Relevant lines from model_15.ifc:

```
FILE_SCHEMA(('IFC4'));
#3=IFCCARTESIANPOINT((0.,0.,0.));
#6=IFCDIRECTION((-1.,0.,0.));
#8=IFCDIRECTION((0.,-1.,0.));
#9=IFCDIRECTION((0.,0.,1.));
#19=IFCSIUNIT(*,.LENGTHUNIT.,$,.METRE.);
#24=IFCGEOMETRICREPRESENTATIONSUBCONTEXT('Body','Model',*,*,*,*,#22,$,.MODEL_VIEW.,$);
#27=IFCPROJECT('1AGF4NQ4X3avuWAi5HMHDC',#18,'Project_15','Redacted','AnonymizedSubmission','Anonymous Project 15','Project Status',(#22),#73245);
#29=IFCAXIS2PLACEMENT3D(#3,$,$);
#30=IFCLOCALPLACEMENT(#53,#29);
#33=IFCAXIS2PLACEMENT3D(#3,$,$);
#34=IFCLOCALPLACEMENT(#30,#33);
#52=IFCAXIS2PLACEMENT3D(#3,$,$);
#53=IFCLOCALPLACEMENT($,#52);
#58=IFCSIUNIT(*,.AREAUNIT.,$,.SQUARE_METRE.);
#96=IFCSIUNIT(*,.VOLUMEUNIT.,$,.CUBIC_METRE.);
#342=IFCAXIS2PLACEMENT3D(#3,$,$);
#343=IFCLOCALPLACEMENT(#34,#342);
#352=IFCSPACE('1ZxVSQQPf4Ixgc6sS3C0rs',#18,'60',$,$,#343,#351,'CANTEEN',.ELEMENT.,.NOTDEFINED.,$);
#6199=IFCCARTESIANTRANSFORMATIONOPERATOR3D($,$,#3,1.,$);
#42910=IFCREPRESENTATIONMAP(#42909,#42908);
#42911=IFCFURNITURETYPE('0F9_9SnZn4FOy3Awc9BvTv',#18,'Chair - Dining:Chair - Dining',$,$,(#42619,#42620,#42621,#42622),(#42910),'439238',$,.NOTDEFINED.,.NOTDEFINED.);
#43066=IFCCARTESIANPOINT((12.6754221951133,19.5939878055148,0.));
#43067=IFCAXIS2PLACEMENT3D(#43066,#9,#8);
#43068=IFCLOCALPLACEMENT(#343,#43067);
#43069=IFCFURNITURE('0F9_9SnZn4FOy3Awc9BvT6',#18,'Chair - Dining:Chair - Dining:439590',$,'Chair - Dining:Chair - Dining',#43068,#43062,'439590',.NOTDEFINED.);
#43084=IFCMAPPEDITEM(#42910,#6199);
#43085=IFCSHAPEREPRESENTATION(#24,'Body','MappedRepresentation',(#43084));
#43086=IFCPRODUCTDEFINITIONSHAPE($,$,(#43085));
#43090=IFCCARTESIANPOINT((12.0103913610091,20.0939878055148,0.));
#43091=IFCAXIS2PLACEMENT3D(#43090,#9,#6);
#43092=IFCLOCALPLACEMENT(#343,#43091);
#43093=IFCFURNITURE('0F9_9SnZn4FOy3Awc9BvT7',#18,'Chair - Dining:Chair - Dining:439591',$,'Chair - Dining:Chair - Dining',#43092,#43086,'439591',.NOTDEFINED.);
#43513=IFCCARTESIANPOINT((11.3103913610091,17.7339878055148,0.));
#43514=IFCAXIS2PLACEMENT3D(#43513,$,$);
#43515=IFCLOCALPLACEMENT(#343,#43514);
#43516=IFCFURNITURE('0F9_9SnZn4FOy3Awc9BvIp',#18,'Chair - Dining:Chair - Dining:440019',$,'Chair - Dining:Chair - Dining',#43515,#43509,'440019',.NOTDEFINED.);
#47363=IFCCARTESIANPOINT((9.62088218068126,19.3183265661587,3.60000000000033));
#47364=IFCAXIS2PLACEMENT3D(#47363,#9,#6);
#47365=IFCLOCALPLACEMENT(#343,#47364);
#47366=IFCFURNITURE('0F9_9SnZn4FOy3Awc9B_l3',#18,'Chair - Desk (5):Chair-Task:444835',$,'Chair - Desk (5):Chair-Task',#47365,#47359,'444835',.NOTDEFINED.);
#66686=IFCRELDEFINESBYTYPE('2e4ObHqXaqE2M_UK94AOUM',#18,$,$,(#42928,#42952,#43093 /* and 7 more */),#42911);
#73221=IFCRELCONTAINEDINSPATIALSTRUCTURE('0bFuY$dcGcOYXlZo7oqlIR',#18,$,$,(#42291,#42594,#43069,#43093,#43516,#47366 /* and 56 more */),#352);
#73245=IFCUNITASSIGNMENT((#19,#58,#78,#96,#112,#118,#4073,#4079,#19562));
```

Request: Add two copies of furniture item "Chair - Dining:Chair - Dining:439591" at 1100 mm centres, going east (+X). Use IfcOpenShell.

```python
import numpy as np
import ifcopenshell
import ifcopenshell.api.geometry
import ifcopenshell.api.root
import ifcopenshell.util.element
import ifcopenshell.util.placement
import ifcopenshell.util.unit

model = ifcopenshell.open("model_15.ifc")
unit_scale = ifcopenshell.util.unit.calculate_unit_scale(model)


def reuse_history(source, copy):
    """copy_class also copies each property set's owner history, people and application; keep the originals."""
    for rel in copy.IsDefinedBy:
        if rel.is_a("IfcRelDefinesByProperties") and (history := rel.RelatingPropertyDefinition.OwnerHistory):
            rel.RelatingPropertyDefinition.OwnerHistory = source.OwnerHistory
            ifcopenshell.util.element.remove_deep2(model, history)


source = model.by_guid("0F9_9SnZn4FOy3Awc9BvT7")
base = ifcopenshell.util.placement.get_local_placement(source.ObjectPlacement)
step = np.array([1.0, 0.0, 0.0]) * 1.1 / unit_scale

for i in range(1, 3):
    copy = ifcopenshell.api.root.copy_class(model, product=source)
    copy.Representation = ifcopenshell.util.element.copy_deep(
        model, source.Representation, exclude=["IfcGeometricRepresentationContext", "IfcRepresentationMap"]
    )
    copy.Name = "Chair - Dining:Chair - Dining"
    copy.Tag = None
    reuse_history(source, copy)
    matrix = base.copy()
    matrix[:3, 3] += i * step
    print("added at", matrix[:3, 3].round(3) + 0.0)
    ifcopenshell.api.geometry.edit_object_placement(model, product=copy, matrix=matrix, is_si=False)

model.write("model_15_edited.ifc")
```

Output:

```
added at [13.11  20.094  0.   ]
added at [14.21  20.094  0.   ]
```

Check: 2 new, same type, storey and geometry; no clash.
